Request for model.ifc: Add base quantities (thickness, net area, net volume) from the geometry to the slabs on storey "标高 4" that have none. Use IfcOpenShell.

First a look at what the model holds.

```python
import ifcopenshell
import ifcopenshell.util.element
import ifcopenshell.util.unit

model = ifcopenshell.open("model.ifc")
print(model.schema)
for unit_type in ("LENGTHUNIT", "AREAUNIT", "VOLUMEUNIT"):
    print(unit_type, ifcopenshell.util.unit.calculate_unit_scale(model, unit_type))
storey = next(s for s in model.by_type("IfcBuildingStorey") if s.Name == "标高 4")
slabs = [e for e in ifcopenshell.util.element.get_decomposition(storey) if e.is_a("IfcSlab")]
for e in sorted(slabs, key=lambda e: e.id()):
    print(e.id(), e.is_a(), e.Name, list(ifcopenshell.util.element.get_psets(e, qtos_only=True)), sep=" | ")
```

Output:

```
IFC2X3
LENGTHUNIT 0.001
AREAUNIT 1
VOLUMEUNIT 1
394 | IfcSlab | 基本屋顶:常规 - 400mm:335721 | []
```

```python
import ifcopenshell
import ifcopenshell.api.pset
import ifcopenshell.geom
import ifcopenshell.util.element
import ifcopenshell.util.shape
import ifcopenshell.util.unit

model = ifcopenshell.open("model.ifc")
unit_scale = ifcopenshell.util.unit.calculate_unit_scale(model)
area_scale = ifcopenshell.util.unit.calculate_unit_scale(model, "AREAUNIT")
volume_scale = ifcopenshell.util.unit.calculate_unit_scale(model, "VOLUMEUNIT")
settings = ifcopenshell.geom.settings()

storey = next(s for s in model.by_type("IfcBuildingStorey") if s.Name == "标高 4")
slabs = [e for e in ifcopenshell.util.element.get_decomposition(storey) if e.is_a("IfcSlab")]

for e in sorted(slabs, key=lambda e: e.id()):
    if ifcopenshell.util.element.get_psets(e, qtos_only=True, should_inherit=False):
        continue
    # Geometry comes back in metres, in the element's own axes.
    shape = ifcopenshell.geom.create_shape(settings, e)
    values = {
        "Width": ifcopenshell.util.shape.get_z(shape.geometry) / unit_scale,
        "NetArea": ifcopenshell.util.shape.get_footprint_area(shape.geometry) / area_scale,
        "NetVolume": ifcopenshell.util.shape.get_volume(shape.geometry) / volume_scale,
    }
    qto = ifcopenshell.api.pset.add_qto(model, product=e, name="BaseQuantities")
    ifcopenshell.api.pset.edit_qto(model, qto=qto, properties=values)
    print(e.id(), {k: round(v, 3) for k, v in values.items()})

model.write("model_updated.ifc")
```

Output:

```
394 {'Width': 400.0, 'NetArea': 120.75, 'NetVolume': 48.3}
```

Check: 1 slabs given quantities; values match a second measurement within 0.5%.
